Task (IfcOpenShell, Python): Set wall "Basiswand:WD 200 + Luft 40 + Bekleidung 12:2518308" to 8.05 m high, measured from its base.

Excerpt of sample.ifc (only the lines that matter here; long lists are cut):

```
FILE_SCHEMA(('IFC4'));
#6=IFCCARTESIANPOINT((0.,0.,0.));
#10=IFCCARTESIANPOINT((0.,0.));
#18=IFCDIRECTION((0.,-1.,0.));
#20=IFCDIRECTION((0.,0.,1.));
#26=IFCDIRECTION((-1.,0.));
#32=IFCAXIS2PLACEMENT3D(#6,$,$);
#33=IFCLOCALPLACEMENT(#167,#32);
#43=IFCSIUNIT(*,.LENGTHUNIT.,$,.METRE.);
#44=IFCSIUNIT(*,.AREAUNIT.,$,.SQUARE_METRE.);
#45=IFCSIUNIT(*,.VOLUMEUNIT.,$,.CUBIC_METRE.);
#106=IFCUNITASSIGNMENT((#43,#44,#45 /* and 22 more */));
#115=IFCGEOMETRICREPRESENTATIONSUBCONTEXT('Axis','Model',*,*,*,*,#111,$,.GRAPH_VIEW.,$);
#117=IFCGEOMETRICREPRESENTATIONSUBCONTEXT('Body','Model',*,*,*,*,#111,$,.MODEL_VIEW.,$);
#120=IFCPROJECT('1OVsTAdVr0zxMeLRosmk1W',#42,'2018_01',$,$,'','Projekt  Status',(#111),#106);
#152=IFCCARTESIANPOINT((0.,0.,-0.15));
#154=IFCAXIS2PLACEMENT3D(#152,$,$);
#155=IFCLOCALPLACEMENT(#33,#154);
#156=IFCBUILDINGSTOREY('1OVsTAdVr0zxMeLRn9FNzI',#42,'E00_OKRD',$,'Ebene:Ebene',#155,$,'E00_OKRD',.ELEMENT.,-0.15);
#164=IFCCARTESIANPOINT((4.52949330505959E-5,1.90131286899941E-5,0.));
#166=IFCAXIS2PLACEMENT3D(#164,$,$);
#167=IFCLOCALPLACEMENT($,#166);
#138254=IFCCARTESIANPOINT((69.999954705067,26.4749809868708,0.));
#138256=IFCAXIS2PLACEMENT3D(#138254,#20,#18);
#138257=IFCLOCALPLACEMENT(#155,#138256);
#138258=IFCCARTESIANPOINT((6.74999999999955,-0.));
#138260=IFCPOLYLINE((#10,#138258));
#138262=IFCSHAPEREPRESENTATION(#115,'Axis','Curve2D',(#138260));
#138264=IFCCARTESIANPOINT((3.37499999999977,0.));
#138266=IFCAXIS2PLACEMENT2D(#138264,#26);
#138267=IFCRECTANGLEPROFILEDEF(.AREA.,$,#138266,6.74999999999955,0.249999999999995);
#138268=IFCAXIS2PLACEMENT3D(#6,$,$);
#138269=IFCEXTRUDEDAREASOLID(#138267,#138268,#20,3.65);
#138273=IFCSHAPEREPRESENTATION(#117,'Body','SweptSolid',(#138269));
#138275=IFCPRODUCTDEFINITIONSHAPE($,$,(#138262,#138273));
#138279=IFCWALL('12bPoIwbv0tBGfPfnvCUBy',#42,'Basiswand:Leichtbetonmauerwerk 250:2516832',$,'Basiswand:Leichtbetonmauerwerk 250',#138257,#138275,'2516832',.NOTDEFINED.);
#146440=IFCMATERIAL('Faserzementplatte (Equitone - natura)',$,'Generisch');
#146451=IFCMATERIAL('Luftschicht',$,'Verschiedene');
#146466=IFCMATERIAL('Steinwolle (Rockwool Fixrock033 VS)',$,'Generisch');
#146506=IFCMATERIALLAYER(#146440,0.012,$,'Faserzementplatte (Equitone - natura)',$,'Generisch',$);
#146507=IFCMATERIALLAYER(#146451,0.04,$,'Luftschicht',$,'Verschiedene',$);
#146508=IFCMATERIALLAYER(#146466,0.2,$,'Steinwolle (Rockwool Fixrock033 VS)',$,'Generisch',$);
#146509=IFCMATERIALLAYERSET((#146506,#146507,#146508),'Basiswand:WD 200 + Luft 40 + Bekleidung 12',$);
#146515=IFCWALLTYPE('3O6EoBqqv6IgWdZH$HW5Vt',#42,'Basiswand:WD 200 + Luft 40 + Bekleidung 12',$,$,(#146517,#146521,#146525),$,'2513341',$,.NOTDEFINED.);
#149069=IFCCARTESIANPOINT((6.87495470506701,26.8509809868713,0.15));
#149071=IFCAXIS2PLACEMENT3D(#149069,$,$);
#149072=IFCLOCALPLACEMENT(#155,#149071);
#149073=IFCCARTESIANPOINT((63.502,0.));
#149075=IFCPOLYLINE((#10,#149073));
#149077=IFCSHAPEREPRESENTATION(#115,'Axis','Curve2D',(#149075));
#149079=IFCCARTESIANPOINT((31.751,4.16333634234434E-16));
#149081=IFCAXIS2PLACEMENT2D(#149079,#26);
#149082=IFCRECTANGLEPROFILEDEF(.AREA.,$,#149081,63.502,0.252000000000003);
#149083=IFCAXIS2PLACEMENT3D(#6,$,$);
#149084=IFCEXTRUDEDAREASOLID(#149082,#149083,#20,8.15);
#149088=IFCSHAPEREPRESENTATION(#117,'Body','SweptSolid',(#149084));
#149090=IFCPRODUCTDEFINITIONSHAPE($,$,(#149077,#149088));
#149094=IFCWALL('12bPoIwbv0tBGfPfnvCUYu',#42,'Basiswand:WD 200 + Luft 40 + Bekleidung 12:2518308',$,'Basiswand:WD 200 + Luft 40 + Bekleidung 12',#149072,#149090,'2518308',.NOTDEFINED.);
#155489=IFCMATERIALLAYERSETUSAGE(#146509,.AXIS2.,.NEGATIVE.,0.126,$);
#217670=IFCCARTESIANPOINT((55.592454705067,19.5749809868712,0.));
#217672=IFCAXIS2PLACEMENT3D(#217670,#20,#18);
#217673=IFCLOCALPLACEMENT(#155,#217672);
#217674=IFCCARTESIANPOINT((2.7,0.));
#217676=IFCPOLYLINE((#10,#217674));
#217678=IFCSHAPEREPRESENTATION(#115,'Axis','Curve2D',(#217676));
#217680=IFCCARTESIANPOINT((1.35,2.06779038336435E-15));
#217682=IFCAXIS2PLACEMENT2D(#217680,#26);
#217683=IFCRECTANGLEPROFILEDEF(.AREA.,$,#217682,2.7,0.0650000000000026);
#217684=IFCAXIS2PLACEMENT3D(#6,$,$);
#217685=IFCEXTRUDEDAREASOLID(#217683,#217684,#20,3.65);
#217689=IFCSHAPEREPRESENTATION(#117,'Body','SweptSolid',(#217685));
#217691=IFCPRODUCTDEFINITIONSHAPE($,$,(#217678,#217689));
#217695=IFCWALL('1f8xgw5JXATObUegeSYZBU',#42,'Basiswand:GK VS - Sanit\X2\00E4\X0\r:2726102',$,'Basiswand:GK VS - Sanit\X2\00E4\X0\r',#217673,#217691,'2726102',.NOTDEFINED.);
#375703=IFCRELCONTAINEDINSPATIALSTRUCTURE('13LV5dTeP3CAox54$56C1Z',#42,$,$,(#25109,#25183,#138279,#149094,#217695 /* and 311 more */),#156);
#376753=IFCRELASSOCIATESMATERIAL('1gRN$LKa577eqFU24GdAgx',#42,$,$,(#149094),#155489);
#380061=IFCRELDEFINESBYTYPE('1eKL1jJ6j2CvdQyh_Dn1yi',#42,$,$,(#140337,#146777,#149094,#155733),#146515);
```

```python
import ifcopenshell
import ifcopenshell.geom
import ifcopenshell.util.representation
import ifcopenshell.util.shape

model = ifcopenshell.open("sample.ifc")
settings = ifcopenshell.geom.settings()


def volume(element):
    """Net volume in cubic metres, openings subtracted."""
    shape = ifcopenshell.geom.create_shape(settings, element)
    return ifcopenshell.util.shape.get_volume(shape.geometry)


wall = model.by_id(149094)
before = volume(wall)

body = ifcopenshell.util.representation.get_representation(wall, "Model", "Body")
solid = body.Items[0]
old_height = solid.Depth
solid.Depth = 8.05
after = volume(wall)

print(f"height {old_height:g} -> {solid.Depth:g}, volume {before:.3f} -> {after:.3f} m3")

model.write("sample_updated.ifc")
```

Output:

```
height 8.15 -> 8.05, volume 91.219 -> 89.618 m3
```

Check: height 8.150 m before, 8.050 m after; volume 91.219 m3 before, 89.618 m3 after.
